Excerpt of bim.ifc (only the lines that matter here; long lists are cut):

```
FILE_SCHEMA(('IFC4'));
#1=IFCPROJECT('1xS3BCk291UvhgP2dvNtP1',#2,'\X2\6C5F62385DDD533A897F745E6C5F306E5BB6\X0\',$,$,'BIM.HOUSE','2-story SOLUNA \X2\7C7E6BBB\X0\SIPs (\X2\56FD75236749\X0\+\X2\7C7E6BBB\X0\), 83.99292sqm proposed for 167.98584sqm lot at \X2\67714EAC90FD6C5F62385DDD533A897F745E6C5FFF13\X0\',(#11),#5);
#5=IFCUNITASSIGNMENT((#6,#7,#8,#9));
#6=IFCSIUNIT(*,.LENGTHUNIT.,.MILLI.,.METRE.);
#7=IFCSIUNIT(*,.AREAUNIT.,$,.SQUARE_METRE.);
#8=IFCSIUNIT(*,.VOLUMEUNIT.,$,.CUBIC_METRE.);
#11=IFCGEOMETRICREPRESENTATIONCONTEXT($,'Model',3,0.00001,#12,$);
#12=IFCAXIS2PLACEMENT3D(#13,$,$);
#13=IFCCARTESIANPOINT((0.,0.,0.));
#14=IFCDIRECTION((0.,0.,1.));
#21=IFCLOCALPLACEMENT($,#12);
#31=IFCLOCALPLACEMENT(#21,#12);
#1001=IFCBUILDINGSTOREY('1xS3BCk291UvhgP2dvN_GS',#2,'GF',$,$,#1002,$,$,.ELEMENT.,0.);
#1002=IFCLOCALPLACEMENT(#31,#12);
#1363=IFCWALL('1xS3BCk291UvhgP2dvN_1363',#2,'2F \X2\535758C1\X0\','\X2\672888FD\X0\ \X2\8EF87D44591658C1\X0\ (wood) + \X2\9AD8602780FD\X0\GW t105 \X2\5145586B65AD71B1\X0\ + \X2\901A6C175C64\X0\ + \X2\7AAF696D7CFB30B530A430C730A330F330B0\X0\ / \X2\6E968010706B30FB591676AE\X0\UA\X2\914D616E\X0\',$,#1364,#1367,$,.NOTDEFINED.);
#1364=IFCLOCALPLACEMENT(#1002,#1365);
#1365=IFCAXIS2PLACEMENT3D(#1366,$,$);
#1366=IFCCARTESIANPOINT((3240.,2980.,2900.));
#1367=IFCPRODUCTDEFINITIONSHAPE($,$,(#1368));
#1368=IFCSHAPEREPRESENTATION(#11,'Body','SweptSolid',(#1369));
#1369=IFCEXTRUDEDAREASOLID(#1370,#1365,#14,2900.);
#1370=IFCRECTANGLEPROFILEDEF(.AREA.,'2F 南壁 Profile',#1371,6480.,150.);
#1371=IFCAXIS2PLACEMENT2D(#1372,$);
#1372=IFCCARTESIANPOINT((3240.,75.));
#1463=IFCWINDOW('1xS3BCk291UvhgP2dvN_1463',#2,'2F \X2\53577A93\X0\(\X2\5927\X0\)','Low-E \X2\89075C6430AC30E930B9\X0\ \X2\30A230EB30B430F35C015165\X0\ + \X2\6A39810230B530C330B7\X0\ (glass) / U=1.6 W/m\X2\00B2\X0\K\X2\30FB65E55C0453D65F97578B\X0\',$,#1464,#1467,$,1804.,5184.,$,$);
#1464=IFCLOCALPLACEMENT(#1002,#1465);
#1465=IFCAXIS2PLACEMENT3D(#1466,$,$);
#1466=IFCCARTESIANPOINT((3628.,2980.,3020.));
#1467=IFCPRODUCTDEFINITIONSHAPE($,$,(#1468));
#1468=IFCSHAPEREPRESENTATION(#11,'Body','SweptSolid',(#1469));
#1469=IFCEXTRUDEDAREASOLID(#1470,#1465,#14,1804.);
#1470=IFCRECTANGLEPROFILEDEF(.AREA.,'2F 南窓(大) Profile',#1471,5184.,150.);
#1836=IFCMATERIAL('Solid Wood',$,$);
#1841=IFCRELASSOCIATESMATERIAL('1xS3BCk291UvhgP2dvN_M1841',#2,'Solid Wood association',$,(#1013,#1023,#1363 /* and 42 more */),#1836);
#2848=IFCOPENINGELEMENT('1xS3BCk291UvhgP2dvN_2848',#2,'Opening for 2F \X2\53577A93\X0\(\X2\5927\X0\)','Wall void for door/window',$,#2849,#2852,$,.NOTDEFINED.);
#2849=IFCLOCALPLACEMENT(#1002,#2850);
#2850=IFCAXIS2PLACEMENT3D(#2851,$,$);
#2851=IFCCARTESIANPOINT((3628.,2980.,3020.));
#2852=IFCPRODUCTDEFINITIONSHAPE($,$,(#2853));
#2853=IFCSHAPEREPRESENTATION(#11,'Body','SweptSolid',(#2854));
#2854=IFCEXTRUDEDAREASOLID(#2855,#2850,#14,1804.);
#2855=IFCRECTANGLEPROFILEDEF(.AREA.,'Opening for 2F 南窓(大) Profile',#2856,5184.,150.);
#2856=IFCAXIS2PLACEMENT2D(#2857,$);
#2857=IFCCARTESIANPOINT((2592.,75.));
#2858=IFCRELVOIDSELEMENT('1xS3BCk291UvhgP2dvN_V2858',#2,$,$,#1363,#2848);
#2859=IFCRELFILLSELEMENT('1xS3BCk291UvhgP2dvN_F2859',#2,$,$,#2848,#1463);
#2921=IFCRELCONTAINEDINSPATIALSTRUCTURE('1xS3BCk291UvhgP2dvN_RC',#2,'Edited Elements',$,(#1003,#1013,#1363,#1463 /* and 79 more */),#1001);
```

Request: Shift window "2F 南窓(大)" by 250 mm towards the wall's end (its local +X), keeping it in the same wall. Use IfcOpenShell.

```python
import ifcopenshell
import ifcopenshell.api.geometry
import ifcopenshell.util.placement
import ifcopenshell.util.unit

model = ifcopenshell.open("bim.ifc")
unit_scale = ifcopenshell.util.unit.calculate_unit_scale(model)

window = model.by_guid("1xS3BCk291UvhgP2dvN_1463")
opening = window.FillsVoids[0].RelatingOpeningElement
wall = opening.VoidsElements[0].RelatingBuildingElement

wall_matrix = ifcopenshell.util.placement.get_local_placement(wall.ObjectPlacement)
shift = wall_matrix[:3, 0] * 0.25 / unit_scale
before = ifcopenshell.util.placement.get_local_placement(window.ObjectPlacement)[:3, 3].copy()

# The window is not placed relative to its opening, so move both.
for product in (opening, window):
    matrix = ifcopenshell.util.placement.get_local_placement(product.ObjectPlacement)
    matrix[:3, 3] += shift
    ifcopenshell.api.geometry.edit_object_placement(model, product=product, matrix=matrix, is_si=False)

after = ifcopenshell.util.placement.get_local_placement(window.ObjectPlacement)[:3, 3]
print("window moved by", (after - before).round(3) + 0.0)

model.write("bim_rev.ifc")
```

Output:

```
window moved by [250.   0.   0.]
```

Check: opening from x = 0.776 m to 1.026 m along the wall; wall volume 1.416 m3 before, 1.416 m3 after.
